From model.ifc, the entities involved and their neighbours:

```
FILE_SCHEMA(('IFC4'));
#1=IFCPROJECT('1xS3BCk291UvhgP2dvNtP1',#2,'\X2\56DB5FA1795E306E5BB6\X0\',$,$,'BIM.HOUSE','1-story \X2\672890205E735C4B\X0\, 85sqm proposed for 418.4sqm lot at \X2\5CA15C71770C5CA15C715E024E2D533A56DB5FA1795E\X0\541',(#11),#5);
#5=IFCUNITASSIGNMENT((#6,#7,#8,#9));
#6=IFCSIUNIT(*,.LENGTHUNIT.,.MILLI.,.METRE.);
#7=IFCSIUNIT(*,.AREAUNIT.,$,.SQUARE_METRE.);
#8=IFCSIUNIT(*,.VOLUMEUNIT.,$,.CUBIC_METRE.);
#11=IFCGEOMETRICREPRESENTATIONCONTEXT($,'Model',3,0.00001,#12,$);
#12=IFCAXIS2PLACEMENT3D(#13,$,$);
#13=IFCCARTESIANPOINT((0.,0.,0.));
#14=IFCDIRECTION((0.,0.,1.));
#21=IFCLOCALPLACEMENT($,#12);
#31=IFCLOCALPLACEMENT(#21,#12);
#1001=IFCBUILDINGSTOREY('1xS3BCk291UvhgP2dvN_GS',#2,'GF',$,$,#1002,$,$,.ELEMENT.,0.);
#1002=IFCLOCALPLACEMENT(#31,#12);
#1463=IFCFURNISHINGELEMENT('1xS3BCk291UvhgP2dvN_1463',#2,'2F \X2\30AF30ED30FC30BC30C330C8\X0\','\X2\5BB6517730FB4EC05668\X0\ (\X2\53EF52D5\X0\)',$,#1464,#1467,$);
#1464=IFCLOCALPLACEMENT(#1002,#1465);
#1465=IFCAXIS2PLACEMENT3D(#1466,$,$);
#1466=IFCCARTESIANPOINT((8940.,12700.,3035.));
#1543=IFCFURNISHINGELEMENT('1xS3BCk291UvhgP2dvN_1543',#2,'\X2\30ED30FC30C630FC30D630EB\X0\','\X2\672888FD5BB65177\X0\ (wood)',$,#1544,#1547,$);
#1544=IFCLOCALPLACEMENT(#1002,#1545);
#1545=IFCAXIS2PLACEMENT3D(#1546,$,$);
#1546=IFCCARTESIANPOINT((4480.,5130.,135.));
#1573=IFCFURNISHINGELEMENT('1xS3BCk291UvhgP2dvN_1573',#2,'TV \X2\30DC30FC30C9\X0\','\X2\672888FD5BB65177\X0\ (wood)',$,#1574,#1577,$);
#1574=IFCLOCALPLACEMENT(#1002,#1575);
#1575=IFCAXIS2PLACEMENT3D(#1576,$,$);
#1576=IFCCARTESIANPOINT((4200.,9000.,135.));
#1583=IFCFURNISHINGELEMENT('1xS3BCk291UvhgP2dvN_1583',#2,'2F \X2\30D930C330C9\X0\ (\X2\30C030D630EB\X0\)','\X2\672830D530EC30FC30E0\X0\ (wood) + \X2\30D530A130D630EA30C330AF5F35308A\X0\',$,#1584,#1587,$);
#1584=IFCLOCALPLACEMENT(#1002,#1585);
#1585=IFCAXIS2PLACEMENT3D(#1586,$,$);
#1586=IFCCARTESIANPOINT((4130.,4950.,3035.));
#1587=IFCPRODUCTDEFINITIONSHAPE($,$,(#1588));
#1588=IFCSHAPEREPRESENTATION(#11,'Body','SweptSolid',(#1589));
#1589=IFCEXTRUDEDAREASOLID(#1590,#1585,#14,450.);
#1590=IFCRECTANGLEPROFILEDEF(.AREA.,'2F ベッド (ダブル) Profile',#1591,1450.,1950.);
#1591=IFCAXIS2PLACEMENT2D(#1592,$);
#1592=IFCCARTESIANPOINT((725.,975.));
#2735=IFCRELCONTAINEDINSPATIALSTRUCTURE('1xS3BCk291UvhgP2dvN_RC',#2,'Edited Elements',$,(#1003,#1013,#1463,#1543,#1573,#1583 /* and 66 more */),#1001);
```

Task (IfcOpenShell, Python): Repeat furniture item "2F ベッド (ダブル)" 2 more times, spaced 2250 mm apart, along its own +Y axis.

```python
import ifcopenshell
import ifcopenshell.api.geometry
import ifcopenshell.api.root
import ifcopenshell.util.element
import ifcopenshell.util.placement

model = ifcopenshell.open("model.ifc")


def reuse_history(source, copy):
    """copy_class also copies each property set's owner history, people and application; keep the originals."""
    for rel in copy.IsDefinedBy:
        if rel.is_a("IfcRelDefinesByProperties") and (history := rel.RelatingPropertyDefinition.OwnerHistory):
            rel.RelatingPropertyDefinition.OwnerHistory = source.OwnerHistory
            ifcopenshell.util.element.remove_deep2(model, history)


source = model.by_guid("1xS3BCk291UvhgP2dvN_1583")
base = ifcopenshell.util.placement.get_local_placement(source.ObjectPlacement)
step = base[:3, 1] * 2250.0

for i in range(1, 3):
    copy = ifcopenshell.api.root.copy_class(model, product=source)
    copy.Representation = ifcopenshell.util.element.copy_deep(
        model, source.Representation, exclude=["IfcGeometricRepresentationContext", "IfcRepresentationMap"]
    )
    reuse_history(source, copy)
    matrix = base.copy()
    matrix[:3, 3] += i * step
    print("added at", matrix[:3, 3].round(3) + 0.0)
    ifcopenshell.api.geometry.edit_object_placement(model, product=copy, matrix=matrix, is_si=False)

model.write("model_rev.ifc")
```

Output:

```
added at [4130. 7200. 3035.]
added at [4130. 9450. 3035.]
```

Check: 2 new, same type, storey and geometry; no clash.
